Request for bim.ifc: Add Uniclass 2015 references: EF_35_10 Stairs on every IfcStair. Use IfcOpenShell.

First a look at what the model holds.

```python
import ifcopenshell

model = ifcopenshell.open("bim.ifc")
print(model.schema)
print("classifications:", [c.Name for c in model.by_type("IfcClassification")])
for ifc_class in ("IfcDoor", "IfcRoof", "IfcStair", "IfcWall", "IfcWindow"):
    print(ifc_class, len(model.by_type(ifc_class)))
```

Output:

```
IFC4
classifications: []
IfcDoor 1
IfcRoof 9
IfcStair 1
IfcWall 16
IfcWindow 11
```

```python
import ifcopenshell
import ifcopenshell.api.classification

model = ifcopenshell.open("bim.ifc")

system = ifcopenshell.api.classification.add_classification(model, classification="Uniclass 2015")

codes = {
    "IfcStair": ("EF_35_10", "Stairs"),
}
for ifc_class, (code, name) in codes.items():
    products = model.by_type(ifc_class)
    ifcopenshell.api.classification.add_reference(
        model, products=products, classification=system, identification=code, name=name
    )
    print(code, len(products))

model.write("bim_edited.ifc")
```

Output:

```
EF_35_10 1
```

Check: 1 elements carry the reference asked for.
